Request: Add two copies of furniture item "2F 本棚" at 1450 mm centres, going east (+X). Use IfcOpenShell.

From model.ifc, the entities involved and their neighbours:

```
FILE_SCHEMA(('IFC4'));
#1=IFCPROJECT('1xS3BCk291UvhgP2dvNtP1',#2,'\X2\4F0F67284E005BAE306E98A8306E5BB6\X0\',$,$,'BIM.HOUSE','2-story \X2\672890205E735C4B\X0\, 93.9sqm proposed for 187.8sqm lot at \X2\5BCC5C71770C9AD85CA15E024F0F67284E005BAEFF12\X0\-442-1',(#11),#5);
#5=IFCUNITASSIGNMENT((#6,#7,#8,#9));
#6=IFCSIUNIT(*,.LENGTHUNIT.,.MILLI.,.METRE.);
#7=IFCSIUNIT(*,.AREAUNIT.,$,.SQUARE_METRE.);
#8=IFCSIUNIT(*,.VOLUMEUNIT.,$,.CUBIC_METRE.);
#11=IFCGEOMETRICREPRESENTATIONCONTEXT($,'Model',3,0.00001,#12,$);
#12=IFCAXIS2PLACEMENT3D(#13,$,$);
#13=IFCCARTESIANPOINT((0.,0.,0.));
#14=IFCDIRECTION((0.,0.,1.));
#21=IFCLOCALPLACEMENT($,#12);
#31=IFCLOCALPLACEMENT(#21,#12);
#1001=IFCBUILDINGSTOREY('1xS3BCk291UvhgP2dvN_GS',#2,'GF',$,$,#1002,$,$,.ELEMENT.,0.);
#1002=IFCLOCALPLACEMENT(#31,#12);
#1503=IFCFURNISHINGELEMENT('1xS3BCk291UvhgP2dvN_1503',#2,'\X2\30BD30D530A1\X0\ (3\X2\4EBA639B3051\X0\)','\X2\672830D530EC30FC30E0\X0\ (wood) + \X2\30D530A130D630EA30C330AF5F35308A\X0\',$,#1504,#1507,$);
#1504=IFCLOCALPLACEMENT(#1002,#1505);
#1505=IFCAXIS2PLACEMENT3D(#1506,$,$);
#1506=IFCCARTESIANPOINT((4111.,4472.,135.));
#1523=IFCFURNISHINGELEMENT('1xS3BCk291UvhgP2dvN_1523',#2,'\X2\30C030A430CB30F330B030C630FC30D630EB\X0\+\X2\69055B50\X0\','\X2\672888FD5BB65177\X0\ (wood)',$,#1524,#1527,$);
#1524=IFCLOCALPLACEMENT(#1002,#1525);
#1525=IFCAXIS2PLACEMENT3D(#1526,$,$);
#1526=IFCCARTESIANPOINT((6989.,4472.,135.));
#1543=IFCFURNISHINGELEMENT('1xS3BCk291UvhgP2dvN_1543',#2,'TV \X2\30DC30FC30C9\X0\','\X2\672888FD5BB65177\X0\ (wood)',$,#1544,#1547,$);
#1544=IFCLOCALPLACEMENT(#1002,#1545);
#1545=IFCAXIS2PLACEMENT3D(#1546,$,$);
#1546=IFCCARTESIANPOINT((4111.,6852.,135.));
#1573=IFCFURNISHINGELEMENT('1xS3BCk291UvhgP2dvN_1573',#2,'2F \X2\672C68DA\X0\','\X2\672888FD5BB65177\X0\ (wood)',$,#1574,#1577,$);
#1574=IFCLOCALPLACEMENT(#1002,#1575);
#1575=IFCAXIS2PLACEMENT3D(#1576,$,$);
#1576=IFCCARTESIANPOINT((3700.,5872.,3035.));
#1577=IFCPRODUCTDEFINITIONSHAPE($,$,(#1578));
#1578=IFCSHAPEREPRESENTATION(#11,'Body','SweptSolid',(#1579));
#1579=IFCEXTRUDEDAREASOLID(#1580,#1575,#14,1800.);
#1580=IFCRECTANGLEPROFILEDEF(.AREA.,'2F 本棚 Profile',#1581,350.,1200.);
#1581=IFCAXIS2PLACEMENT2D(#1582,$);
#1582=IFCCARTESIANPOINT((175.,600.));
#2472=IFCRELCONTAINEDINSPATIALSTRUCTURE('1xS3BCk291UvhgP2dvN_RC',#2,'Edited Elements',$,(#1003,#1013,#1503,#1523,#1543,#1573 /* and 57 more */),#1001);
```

```python
import numpy as np
import ifcopenshell
import ifcopenshell.api.geometry
import ifcopenshell.api.root
import ifcopenshell.util.element
import ifcopenshell.util.placement

model = ifcopenshell.open("model.ifc")


def reuse_history(source, copy):
    """copy_class also copies each property set's owner history, people and application; keep the originals."""
    for rel in copy.IsDefinedBy:
        if rel.is_a("IfcRelDefinesByProperties") and (history := rel.RelatingPropertyDefinition.OwnerHistory):
            rel.RelatingPropertyDefinition.OwnerHistory = source.OwnerHistory
            ifcopenshell.util.element.remove_deep2(model, history)


source = model.by_id(1573)
base = ifcopenshell.util.placement.get_local_placement(source.ObjectPlacement)
step = np.array([1.0, 0.0, 0.0]) * 1450.0

for i in range(1, 3):
    copy = ifcopenshell.api.root.copy_class(model, product=source)
    copy.Representation = ifcopenshell.util.element.copy_deep(
        model, source.Representation, exclude=["IfcGeometricRepresentationContext", "IfcRepresentationMap"]
    )
    reuse_history(source, copy)
    matrix = base.copy()
    matrix[:3, 3] += i * step
    print("added at", matrix[:3, 3].round(3) + 0.0)
    ifcopenshell.api.geometry.edit_object_placement(model, product=copy, matrix=matrix, is_si=False)

model.write("model-out.ifc")
```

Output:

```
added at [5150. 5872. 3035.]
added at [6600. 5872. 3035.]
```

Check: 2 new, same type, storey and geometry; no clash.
